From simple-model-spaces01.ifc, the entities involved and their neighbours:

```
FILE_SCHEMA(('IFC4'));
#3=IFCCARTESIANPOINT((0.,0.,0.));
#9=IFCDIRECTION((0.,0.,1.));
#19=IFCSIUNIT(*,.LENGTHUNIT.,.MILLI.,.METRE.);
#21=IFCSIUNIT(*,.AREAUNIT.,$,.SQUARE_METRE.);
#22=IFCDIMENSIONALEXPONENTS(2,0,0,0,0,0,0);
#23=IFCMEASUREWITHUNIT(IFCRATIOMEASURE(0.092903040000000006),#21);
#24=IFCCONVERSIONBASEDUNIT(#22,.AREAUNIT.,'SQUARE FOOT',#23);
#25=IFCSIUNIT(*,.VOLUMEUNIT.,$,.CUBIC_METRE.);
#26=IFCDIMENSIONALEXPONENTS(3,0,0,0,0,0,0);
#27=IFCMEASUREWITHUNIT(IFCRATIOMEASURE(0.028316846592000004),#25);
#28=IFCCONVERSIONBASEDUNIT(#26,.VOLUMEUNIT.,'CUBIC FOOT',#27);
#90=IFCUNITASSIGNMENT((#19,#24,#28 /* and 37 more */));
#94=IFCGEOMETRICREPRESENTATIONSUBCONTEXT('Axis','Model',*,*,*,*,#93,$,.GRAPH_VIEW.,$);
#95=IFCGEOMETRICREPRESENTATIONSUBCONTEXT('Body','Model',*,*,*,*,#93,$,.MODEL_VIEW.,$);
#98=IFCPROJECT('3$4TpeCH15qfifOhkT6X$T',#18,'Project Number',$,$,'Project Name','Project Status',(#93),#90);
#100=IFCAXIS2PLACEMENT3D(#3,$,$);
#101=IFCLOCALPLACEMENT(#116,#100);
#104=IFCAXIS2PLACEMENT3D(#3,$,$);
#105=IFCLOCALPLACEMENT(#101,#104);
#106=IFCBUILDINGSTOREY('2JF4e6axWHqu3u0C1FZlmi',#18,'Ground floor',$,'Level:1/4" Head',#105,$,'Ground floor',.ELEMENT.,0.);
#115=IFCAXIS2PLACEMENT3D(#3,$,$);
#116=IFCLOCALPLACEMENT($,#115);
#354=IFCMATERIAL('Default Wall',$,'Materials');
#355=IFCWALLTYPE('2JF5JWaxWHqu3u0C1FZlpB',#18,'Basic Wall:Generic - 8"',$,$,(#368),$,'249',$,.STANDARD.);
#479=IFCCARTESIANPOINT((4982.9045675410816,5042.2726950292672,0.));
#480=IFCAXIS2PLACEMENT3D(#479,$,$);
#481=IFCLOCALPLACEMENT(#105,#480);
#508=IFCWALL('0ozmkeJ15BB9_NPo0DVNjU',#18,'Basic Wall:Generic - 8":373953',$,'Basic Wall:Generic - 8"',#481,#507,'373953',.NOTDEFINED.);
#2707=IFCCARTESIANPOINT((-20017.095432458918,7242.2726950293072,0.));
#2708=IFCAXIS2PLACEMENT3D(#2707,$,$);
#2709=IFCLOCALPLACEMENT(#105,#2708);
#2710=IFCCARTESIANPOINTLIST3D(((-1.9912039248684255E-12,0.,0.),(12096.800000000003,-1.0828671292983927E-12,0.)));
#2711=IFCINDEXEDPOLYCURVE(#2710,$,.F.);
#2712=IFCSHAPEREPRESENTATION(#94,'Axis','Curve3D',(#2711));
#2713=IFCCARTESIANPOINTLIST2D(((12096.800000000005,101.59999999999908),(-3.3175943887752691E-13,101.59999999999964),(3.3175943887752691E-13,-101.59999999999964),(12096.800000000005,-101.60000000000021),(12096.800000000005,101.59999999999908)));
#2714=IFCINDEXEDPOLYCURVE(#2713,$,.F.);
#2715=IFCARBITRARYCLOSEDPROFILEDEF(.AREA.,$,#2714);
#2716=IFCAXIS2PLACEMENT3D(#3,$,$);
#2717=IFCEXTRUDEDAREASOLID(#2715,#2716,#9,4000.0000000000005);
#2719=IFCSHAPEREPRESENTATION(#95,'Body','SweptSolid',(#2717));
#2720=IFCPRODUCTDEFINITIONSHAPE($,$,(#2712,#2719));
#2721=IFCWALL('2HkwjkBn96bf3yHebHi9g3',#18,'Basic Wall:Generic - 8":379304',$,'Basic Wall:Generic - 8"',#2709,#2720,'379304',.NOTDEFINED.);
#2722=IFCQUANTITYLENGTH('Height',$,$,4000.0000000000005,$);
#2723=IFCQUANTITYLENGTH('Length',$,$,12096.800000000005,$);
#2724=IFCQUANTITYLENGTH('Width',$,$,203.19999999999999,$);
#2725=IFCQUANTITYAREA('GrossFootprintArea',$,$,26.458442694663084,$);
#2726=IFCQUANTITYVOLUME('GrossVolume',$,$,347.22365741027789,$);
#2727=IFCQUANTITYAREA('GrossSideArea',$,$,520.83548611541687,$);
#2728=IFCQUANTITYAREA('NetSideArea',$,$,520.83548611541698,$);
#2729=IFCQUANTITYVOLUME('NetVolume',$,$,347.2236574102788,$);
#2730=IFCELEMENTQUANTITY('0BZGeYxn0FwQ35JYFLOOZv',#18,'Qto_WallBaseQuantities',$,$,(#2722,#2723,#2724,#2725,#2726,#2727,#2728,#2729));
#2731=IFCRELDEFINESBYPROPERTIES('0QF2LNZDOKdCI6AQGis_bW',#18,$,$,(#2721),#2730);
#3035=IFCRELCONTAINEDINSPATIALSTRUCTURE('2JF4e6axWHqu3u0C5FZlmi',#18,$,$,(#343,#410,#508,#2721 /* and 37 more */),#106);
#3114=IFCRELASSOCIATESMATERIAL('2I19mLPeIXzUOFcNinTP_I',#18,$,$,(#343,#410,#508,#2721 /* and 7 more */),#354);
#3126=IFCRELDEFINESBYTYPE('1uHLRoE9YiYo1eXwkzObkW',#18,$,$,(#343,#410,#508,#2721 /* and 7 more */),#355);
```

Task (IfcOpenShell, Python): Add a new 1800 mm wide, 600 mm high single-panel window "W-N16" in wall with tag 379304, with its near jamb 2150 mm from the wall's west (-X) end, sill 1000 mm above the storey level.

```python
import numpy as np
import ifcopenshell
import ifcopenshell.api.feature
import ifcopenshell.api.geometry
import ifcopenshell.api.pset
import ifcopenshell.api.root
import ifcopenshell.api.spatial
import ifcopenshell.geom
import ifcopenshell.util.element
import ifcopenshell.util.placement
import ifcopenshell.util.representation
import ifcopenshell.util.shape
import ifcopenshell.util.unit

model = ifcopenshell.open("simple-model-spaces01.ifc")
unit_scale = ifcopenshell.util.unit.calculate_unit_scale(model)
area_scale = ifcopenshell.util.unit.calculate_unit_scale(model, "AREAUNIT")
volume_scale = ifcopenshell.util.unit.calculate_unit_scale(model, "VOLUMEUNIT")
settings = ifcopenshell.geom.settings()


def volume(element):
    """Net volume in cubic metres, openings subtracted."""
    shape = ifcopenshell.geom.create_shape(settings, element)
    return ifcopenshell.util.shape.get_volume(shape.geometry)


wall = model.by_id(2721)
storey = ifcopenshell.util.element.get_container(wall, ifc_class="IfcBuildingStorey")
context = ifcopenshell.util.representation.get_context(model, "Model", "Body", "MODEL_VIEW")
before = volume(wall)

width, height, from_end, sill = 1.8, 0.6, 2.15, 1  # metres

# The wall runs along its own X axis, and the end named is its -X end.
wall_shape = ifcopenshell.geom.create_shape(settings, wall)
x, y, z = ifcopenshell.util.shape.get_vertices(wall_shape.geometry).T
start = x.min() + from_end
face, thickness = float(y.min()), float(y.max() - y.min())
wall_matrix = ifcopenshell.util.placement.get_local_placement(wall.ObjectPlacement)
level = ifcopenshell.util.placement.get_local_placement(storey.ObjectPlacement)[2, 3]


def in_wall(x, y):
    """Placement at x, y metres in the wall's axes, at sill height."""
    matrix = wall_matrix.copy()
    matrix[:, 3] = wall_matrix @ np.array([x / unit_scale, y / unit_scale, 0.0, 1.0])
    matrix[2, 3] = level + sill / unit_scale
    return matrix


# Opening: a box that overshoots both wall faces by 50 mm.
opening = ifcopenshell.api.root.create_entity(model, ifc_class="IfcOpeningElement", predefined_type="OPENING")
box = ifcopenshell.api.geometry.add_wall_representation(
    model, context=context, length=width, height=height, thickness=thickness + 0.1
)
ifcopenshell.api.geometry.assign_representation(model, product=opening, representation=box)
ifcopenshell.api.geometry.edit_object_placement(model, product=opening, matrix=in_wall(start, face - 0.05), is_si=False)
ifcopenshell.api.feature.add_feature(model, feature=opening, element=wall)

window = ifcopenshell.api.root.create_entity(model, ifc_class="IfcWindow", name="W-N16", predefined_type="WINDOW")
window.OverallWidth, window.OverallHeight = width / unit_scale, height / unit_scale
window.PartitioningType = "SINGLE_PANEL"
body = ifcopenshell.api.geometry.add_window_representation(
    model,
    context=context,
    overall_width=window.OverallWidth,
    overall_height=window.OverallHeight,
    partition_type="SINGLE_PANEL",
)
ifcopenshell.api.geometry.assign_representation(model, product=window, representation=body)
ifcopenshell.api.spatial.assign_container(model, products=[window], relating_structure=storey)
ifcopenshell.api.feature.add_filling(model, opening=opening, element=window)

# Centre the window in the wall's thickness.
ifcopenshell.api.geometry.edit_object_placement(model, product=window, matrix=in_wall(start, face), is_si=False)
window_shape = ifcopenshell.geom.create_shape(settings, window)
depth = ifcopenshell.util.shape.get_vertices(window_shape.geometry)[:, 1]
offset = face + thickness / 2 - (depth.min() + depth.max()) / 2
ifcopenshell.api.geometry.edit_object_placement(model, product=window, matrix=in_wall(start, offset), is_si=False)

after = volume(wall)

# Update the wall's stored quantities.
qto = model.by_id(ifcopenshell.util.element.get_pset(wall, "Qto_WallBaseQuantities", should_inherit=False)["id"])
ifcopenshell.api.pset.edit_qto(model, qto=qto, properties={
    "NetSideArea": after / thickness / area_scale,
    "NetVolume": after / volume_scale,
})

print(f"wall volume {before:.3f} -> {after:.3f} m3")

model.write("simple-model-spaces01_edited.ifc")
```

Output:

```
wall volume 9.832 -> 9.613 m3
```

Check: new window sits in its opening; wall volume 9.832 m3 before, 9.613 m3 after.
